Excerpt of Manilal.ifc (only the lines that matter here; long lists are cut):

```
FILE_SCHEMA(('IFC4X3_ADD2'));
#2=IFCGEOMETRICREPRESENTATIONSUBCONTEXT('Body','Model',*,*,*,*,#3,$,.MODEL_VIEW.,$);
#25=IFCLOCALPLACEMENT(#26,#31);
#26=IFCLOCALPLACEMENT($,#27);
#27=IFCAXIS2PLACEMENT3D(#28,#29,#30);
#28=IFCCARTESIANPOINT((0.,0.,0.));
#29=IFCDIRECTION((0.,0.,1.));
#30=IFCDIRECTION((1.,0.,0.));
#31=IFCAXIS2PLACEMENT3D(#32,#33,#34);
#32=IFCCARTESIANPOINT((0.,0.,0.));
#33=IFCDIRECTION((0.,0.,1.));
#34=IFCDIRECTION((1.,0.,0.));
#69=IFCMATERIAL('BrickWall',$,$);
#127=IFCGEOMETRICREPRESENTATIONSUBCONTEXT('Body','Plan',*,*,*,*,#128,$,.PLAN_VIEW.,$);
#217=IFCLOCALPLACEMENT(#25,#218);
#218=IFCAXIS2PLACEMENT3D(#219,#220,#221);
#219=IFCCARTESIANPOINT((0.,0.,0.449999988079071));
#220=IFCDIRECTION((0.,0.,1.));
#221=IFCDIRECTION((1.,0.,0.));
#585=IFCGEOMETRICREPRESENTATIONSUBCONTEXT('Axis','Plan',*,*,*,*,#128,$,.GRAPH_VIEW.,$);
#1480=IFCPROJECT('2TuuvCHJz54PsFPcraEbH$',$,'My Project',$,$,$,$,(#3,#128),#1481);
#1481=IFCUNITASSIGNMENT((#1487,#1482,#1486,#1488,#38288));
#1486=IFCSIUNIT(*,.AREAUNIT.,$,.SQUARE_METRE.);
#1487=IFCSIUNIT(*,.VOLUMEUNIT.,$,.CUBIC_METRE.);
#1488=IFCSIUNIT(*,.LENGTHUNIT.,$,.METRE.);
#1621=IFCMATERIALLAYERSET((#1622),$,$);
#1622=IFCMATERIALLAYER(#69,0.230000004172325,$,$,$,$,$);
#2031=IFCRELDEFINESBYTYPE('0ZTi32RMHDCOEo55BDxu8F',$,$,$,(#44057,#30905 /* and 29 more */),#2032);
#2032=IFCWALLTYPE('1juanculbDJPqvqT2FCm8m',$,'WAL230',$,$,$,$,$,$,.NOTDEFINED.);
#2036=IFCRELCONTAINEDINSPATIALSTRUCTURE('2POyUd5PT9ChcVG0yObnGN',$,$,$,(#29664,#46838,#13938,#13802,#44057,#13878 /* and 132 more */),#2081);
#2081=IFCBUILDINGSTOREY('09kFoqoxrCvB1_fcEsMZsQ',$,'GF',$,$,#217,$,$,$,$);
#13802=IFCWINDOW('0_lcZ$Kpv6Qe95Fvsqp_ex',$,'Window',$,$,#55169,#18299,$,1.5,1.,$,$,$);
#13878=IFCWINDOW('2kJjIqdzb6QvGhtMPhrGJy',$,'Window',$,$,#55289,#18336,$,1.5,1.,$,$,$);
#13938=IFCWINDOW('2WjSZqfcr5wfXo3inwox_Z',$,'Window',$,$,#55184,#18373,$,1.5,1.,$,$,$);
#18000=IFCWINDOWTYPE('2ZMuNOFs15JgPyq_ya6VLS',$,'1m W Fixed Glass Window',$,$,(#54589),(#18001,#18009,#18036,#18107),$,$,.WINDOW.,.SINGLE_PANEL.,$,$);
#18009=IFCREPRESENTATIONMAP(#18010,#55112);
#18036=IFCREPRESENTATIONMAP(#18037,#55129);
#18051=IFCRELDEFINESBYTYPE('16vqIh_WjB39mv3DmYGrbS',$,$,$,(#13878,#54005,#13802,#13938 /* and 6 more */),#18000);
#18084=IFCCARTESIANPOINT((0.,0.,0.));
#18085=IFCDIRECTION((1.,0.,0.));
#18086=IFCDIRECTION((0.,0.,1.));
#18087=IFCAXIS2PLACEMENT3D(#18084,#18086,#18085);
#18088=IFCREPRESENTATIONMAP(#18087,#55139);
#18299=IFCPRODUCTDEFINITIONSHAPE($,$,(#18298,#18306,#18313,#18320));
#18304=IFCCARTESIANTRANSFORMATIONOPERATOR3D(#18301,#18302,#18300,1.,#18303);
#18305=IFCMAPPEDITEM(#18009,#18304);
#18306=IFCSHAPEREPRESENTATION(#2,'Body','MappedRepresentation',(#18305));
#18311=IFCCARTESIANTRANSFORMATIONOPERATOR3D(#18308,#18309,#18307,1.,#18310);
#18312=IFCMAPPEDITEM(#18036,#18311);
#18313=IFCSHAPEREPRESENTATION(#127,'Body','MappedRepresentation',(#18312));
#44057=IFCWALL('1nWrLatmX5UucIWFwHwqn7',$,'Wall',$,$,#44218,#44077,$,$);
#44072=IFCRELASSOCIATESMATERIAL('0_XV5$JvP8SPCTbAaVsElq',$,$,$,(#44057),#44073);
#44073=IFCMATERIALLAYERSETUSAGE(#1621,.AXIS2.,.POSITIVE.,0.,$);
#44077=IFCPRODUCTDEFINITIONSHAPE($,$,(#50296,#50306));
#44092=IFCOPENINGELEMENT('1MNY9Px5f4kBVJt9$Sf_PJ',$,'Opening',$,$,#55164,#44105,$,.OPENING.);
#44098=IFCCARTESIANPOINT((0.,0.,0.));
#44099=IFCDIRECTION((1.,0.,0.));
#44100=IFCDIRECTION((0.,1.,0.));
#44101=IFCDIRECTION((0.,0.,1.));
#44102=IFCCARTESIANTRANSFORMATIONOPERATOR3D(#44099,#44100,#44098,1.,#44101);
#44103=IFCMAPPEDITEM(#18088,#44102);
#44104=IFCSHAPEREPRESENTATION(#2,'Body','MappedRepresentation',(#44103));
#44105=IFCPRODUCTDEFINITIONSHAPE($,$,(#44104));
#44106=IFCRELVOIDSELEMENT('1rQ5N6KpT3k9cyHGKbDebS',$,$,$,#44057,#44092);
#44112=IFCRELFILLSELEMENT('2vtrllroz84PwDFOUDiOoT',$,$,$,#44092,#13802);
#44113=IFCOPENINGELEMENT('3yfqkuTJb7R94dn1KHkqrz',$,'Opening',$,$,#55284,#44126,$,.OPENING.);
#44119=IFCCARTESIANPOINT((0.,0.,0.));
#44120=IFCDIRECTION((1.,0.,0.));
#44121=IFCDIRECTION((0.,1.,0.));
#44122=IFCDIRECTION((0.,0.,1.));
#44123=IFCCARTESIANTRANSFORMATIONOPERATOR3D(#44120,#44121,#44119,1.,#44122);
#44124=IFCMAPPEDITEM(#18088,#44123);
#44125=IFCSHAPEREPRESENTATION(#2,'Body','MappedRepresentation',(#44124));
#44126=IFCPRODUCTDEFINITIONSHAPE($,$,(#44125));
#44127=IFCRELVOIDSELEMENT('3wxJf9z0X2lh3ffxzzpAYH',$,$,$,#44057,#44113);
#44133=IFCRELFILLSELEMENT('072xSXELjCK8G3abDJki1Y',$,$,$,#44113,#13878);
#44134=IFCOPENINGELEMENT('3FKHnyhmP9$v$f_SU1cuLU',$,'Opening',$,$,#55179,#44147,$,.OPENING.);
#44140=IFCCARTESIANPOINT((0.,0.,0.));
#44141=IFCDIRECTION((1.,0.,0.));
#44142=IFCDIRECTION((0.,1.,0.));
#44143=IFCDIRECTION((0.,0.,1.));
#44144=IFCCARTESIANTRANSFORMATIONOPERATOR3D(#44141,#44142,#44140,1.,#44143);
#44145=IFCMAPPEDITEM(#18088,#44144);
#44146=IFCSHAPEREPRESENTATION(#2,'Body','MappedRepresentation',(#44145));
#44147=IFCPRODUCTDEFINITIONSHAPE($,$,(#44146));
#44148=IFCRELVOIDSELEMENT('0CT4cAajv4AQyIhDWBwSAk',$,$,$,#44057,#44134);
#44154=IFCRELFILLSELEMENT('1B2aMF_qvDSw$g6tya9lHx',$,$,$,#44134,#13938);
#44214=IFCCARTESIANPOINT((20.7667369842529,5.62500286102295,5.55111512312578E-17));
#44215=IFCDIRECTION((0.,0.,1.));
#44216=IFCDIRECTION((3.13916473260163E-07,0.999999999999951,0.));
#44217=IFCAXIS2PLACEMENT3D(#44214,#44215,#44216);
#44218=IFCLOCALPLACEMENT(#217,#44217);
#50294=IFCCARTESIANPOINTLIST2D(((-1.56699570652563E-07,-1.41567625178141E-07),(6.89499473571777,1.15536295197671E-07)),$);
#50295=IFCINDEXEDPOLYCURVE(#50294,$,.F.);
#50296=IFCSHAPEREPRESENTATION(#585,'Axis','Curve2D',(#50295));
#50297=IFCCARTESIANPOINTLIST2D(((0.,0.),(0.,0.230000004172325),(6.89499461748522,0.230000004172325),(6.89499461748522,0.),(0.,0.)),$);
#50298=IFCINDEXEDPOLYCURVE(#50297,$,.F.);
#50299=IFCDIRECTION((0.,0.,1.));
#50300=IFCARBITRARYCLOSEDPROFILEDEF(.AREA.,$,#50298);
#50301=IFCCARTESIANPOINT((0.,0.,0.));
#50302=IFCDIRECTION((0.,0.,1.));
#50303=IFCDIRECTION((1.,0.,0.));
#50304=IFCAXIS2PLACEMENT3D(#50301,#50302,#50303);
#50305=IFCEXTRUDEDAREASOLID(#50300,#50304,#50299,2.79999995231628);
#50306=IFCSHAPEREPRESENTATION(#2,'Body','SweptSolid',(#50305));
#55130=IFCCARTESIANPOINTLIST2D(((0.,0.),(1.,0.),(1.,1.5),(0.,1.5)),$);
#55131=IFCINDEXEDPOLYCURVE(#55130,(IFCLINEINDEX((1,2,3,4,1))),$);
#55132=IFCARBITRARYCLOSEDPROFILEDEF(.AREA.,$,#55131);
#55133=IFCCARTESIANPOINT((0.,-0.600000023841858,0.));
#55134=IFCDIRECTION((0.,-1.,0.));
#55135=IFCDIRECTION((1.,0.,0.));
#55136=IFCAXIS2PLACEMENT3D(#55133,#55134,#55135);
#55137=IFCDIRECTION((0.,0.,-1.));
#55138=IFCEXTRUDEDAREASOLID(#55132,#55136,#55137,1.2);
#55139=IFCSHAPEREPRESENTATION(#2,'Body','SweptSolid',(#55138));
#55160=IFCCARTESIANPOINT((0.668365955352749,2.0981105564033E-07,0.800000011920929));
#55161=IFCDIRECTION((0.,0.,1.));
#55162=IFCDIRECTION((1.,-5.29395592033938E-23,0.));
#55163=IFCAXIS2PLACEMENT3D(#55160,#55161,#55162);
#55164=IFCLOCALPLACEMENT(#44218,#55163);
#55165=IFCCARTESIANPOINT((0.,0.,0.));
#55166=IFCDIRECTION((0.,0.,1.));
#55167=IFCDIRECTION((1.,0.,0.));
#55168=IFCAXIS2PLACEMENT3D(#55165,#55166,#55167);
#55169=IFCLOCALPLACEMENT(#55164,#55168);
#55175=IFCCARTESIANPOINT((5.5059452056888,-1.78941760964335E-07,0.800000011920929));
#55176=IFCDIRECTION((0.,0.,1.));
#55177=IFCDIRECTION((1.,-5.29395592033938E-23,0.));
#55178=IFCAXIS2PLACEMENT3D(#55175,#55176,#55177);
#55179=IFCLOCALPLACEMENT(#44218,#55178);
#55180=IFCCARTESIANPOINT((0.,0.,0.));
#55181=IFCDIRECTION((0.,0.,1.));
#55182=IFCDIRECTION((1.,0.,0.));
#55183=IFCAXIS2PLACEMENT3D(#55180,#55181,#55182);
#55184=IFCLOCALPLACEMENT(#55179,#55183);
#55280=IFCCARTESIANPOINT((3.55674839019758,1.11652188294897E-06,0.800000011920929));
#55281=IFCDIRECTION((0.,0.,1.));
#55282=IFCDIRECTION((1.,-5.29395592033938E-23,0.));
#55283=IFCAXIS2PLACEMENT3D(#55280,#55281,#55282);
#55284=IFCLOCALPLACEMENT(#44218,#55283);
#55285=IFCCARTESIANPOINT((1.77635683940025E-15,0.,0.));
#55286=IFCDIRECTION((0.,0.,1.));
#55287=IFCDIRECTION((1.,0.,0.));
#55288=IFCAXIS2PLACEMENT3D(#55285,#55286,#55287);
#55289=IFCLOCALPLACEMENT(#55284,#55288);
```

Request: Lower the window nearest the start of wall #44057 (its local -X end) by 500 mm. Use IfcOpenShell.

```python
import numpy as np
import ifcopenshell
import ifcopenshell.api.geometry
import ifcopenshell.util.placement
import ifcopenshell.util.unit

model = ifcopenshell.open("Manilal.ifc")
unit_scale = ifcopenshell.util.unit.calculate_unit_scale(model)

window = model.by_id(13802)
opening = window.FillsVoids[0].RelatingOpeningElement
dz = -0.5 / unit_scale

shift = np.array([0.0, 0.0, dz])
# The window is placed relative to its opening, so it follows when the opening moves.
matrix = ifcopenshell.util.placement.get_local_placement(opening.ObjectPlacement)
matrix[:3, 3] += shift
ifcopenshell.api.geometry.edit_object_placement(
    model, product=opening, matrix=matrix, is_si=False, should_transform_children=True
)

print(f"moved by {dz * unit_scale:+.3f} m")

model.write("Manilal_edited.ifc")
```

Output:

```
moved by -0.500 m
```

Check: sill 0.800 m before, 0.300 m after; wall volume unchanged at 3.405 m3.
